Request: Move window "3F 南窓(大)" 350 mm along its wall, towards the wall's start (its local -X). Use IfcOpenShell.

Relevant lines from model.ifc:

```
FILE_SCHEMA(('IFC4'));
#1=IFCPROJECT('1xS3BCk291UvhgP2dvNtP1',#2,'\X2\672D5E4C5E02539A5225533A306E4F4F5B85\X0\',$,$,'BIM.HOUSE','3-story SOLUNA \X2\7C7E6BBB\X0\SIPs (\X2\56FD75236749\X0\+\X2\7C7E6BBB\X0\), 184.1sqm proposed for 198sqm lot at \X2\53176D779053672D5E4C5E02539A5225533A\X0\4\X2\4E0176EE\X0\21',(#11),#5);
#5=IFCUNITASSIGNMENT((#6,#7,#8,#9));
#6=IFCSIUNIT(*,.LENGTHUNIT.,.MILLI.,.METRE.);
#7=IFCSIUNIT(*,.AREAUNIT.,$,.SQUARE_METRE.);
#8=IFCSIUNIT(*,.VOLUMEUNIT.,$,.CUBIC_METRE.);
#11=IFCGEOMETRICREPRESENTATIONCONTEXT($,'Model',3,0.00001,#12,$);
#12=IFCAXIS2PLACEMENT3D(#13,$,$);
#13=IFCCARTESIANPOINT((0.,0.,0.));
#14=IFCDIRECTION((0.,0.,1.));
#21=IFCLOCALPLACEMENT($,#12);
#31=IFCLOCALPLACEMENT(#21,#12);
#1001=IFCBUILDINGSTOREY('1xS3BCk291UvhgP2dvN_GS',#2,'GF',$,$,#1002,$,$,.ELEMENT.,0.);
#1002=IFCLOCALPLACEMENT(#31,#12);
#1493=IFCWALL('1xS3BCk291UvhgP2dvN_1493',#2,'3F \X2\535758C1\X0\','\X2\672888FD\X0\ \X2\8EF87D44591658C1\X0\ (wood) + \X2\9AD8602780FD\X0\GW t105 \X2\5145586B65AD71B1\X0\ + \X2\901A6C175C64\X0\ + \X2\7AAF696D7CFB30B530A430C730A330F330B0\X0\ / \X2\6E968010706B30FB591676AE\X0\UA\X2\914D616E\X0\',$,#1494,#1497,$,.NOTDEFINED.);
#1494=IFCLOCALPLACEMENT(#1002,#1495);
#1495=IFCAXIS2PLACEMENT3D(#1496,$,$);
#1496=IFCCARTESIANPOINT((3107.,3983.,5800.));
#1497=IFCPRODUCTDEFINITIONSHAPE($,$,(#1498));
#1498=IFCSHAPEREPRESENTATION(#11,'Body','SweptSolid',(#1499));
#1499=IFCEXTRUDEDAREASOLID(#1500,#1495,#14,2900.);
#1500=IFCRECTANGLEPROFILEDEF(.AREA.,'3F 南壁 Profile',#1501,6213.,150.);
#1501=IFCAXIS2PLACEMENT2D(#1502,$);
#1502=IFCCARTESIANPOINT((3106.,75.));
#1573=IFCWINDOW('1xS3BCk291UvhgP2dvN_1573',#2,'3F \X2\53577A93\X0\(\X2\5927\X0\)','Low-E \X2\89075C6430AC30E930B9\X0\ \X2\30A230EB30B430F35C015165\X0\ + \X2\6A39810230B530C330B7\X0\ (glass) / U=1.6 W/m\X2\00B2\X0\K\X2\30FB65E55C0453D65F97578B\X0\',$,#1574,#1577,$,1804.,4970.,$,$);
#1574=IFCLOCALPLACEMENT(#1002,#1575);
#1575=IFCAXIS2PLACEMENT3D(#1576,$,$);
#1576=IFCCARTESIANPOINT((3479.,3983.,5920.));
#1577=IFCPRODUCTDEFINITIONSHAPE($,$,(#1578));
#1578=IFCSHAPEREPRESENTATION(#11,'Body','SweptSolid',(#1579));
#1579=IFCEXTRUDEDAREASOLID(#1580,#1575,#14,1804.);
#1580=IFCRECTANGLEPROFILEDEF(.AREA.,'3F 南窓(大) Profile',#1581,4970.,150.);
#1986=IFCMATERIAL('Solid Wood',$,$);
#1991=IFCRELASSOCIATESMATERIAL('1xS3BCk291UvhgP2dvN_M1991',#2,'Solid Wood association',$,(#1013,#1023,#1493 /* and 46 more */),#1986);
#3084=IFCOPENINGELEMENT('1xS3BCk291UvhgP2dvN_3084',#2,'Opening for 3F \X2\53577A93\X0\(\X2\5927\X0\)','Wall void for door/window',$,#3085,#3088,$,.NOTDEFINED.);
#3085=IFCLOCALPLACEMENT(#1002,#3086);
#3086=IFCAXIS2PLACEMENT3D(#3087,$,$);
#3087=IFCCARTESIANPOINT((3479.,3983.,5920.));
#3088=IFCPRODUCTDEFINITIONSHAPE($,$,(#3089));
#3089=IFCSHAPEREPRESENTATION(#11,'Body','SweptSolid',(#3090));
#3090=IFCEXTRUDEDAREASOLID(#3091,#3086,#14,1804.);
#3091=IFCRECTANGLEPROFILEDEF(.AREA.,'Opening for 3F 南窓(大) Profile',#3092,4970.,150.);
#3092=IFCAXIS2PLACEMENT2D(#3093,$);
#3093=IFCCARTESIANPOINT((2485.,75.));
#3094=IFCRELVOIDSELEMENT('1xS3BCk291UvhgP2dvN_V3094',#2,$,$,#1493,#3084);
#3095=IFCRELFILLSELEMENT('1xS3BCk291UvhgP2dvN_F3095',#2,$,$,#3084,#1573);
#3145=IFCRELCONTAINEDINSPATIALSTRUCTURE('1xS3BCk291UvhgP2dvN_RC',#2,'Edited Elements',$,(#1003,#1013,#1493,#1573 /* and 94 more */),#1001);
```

```python
import ifcopenshell
import ifcopenshell.api.geometry
import ifcopenshell.util.placement

model = ifcopenshell.open("model.ifc")

window = model.by_guid("1xS3BCk291UvhgP2dvN_1573")
opening = window.FillsVoids[0].RelatingOpeningElement
wall = opening.VoidsElements[0].RelatingBuildingElement

wall_matrix = ifcopenshell.util.placement.get_local_placement(wall.ObjectPlacement)
shift = wall_matrix[:3, 0] * -350.0
before = ifcopenshell.util.placement.get_local_placement(window.ObjectPlacement)[:3, 3].copy()

# The window is not placed relative to its opening, so move both.
for product in (opening, window):
    matrix = ifcopenshell.util.placement.get_local_placement(product.ObjectPlacement)
    matrix[:3, 3] += shift
    ifcopenshell.api.geometry.edit_object_placement(model, product=product, matrix=matrix, is_si=False)

after = ifcopenshell.util.placement.get_local_placement(window.ObjectPlacement)[:3, 3]
print("window moved by", (after - before).round(3) + 0.0)

model.write("model_updated.ifc")
```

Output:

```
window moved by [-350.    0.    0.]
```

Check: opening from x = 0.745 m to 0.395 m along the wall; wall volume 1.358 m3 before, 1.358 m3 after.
